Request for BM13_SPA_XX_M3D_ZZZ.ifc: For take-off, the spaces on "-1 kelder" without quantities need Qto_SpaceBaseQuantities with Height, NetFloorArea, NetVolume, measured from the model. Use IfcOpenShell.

First a look at what the model holds.

```python
import ifcopenshell
import ifcopenshell.util.element
import ifcopenshell.util.unit

model = ifcopenshell.open("BM13_SPA_XX_M3D_ZZZ.ifc")
print(model.schema)
for unit_type in ("LENGTHUNIT", "AREAUNIT", "VOLUMEUNIT"):
    print(unit_type, ifcopenshell.util.unit.calculate_unit_scale(model, unit_type))
storey = next(s for s in model.by_type("IfcBuildingStorey") if s.Name == "-1 kelder")
spaces = [e for e in ifcopenshell.util.element.get_decomposition(storey) if e.is_a("IfcSpace")]
for e in sorted(spaces, key=lambda e: e.id()):
    print(e.id(), e.is_a(), e.Name, list(ifcopenshell.util.element.get_psets(e, qtos_only=True)), sep=" | ")
```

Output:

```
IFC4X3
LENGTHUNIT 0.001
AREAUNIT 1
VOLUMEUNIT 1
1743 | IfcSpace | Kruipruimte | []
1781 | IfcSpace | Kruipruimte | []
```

```python
import ifcopenshell
import ifcopenshell.api.pset
import ifcopenshell.geom
import ifcopenshell.util.element
import ifcopenshell.util.shape
import ifcopenshell.util.unit

model = ifcopenshell.open("BM13_SPA_XX_M3D_ZZZ.ifc")
unit_scale = ifcopenshell.util.unit.calculate_unit_scale(model)
area_scale = ifcopenshell.util.unit.calculate_unit_scale(model, "AREAUNIT")
volume_scale = ifcopenshell.util.unit.calculate_unit_scale(model, "VOLUMEUNIT")
settings = ifcopenshell.geom.settings()

storey = next(s for s in model.by_type("IfcBuildingStorey") if s.Name == "-1 kelder")
spaces = [e for e in ifcopenshell.util.element.get_decomposition(storey) if e.is_a("IfcSpace")]

for e in sorted(spaces, key=lambda e: e.id()):
    if ifcopenshell.util.element.get_psets(e, qtos_only=True, should_inherit=False):
        continue
    # Geometry comes back in metres, in the element's own axes.
    shape = ifcopenshell.geom.create_shape(settings, e)
    values = {
        "Height": ifcopenshell.util.shape.get_z(shape.geometry) / unit_scale,
        "NetFloorArea": ifcopenshell.util.shape.get_footprint_area(shape.geometry) / area_scale,
        "NetVolume": ifcopenshell.util.shape.get_volume(shape.geometry) / volume_scale,
    }
    qto = ifcopenshell.api.pset.add_qto(model, product=e, name="Qto_SpaceBaseQuantities")
    ifcopenshell.api.pset.edit_qto(model, qto=qto, properties=values)
    print(e.id(), {k: round(v, 3) for k, v in values.items()})

model.write("BM13_SPA_XX_M3D_ZZZ-out.ifc")
```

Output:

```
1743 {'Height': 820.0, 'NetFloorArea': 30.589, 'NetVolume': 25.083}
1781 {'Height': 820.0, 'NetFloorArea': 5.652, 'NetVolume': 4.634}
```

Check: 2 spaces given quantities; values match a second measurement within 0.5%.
